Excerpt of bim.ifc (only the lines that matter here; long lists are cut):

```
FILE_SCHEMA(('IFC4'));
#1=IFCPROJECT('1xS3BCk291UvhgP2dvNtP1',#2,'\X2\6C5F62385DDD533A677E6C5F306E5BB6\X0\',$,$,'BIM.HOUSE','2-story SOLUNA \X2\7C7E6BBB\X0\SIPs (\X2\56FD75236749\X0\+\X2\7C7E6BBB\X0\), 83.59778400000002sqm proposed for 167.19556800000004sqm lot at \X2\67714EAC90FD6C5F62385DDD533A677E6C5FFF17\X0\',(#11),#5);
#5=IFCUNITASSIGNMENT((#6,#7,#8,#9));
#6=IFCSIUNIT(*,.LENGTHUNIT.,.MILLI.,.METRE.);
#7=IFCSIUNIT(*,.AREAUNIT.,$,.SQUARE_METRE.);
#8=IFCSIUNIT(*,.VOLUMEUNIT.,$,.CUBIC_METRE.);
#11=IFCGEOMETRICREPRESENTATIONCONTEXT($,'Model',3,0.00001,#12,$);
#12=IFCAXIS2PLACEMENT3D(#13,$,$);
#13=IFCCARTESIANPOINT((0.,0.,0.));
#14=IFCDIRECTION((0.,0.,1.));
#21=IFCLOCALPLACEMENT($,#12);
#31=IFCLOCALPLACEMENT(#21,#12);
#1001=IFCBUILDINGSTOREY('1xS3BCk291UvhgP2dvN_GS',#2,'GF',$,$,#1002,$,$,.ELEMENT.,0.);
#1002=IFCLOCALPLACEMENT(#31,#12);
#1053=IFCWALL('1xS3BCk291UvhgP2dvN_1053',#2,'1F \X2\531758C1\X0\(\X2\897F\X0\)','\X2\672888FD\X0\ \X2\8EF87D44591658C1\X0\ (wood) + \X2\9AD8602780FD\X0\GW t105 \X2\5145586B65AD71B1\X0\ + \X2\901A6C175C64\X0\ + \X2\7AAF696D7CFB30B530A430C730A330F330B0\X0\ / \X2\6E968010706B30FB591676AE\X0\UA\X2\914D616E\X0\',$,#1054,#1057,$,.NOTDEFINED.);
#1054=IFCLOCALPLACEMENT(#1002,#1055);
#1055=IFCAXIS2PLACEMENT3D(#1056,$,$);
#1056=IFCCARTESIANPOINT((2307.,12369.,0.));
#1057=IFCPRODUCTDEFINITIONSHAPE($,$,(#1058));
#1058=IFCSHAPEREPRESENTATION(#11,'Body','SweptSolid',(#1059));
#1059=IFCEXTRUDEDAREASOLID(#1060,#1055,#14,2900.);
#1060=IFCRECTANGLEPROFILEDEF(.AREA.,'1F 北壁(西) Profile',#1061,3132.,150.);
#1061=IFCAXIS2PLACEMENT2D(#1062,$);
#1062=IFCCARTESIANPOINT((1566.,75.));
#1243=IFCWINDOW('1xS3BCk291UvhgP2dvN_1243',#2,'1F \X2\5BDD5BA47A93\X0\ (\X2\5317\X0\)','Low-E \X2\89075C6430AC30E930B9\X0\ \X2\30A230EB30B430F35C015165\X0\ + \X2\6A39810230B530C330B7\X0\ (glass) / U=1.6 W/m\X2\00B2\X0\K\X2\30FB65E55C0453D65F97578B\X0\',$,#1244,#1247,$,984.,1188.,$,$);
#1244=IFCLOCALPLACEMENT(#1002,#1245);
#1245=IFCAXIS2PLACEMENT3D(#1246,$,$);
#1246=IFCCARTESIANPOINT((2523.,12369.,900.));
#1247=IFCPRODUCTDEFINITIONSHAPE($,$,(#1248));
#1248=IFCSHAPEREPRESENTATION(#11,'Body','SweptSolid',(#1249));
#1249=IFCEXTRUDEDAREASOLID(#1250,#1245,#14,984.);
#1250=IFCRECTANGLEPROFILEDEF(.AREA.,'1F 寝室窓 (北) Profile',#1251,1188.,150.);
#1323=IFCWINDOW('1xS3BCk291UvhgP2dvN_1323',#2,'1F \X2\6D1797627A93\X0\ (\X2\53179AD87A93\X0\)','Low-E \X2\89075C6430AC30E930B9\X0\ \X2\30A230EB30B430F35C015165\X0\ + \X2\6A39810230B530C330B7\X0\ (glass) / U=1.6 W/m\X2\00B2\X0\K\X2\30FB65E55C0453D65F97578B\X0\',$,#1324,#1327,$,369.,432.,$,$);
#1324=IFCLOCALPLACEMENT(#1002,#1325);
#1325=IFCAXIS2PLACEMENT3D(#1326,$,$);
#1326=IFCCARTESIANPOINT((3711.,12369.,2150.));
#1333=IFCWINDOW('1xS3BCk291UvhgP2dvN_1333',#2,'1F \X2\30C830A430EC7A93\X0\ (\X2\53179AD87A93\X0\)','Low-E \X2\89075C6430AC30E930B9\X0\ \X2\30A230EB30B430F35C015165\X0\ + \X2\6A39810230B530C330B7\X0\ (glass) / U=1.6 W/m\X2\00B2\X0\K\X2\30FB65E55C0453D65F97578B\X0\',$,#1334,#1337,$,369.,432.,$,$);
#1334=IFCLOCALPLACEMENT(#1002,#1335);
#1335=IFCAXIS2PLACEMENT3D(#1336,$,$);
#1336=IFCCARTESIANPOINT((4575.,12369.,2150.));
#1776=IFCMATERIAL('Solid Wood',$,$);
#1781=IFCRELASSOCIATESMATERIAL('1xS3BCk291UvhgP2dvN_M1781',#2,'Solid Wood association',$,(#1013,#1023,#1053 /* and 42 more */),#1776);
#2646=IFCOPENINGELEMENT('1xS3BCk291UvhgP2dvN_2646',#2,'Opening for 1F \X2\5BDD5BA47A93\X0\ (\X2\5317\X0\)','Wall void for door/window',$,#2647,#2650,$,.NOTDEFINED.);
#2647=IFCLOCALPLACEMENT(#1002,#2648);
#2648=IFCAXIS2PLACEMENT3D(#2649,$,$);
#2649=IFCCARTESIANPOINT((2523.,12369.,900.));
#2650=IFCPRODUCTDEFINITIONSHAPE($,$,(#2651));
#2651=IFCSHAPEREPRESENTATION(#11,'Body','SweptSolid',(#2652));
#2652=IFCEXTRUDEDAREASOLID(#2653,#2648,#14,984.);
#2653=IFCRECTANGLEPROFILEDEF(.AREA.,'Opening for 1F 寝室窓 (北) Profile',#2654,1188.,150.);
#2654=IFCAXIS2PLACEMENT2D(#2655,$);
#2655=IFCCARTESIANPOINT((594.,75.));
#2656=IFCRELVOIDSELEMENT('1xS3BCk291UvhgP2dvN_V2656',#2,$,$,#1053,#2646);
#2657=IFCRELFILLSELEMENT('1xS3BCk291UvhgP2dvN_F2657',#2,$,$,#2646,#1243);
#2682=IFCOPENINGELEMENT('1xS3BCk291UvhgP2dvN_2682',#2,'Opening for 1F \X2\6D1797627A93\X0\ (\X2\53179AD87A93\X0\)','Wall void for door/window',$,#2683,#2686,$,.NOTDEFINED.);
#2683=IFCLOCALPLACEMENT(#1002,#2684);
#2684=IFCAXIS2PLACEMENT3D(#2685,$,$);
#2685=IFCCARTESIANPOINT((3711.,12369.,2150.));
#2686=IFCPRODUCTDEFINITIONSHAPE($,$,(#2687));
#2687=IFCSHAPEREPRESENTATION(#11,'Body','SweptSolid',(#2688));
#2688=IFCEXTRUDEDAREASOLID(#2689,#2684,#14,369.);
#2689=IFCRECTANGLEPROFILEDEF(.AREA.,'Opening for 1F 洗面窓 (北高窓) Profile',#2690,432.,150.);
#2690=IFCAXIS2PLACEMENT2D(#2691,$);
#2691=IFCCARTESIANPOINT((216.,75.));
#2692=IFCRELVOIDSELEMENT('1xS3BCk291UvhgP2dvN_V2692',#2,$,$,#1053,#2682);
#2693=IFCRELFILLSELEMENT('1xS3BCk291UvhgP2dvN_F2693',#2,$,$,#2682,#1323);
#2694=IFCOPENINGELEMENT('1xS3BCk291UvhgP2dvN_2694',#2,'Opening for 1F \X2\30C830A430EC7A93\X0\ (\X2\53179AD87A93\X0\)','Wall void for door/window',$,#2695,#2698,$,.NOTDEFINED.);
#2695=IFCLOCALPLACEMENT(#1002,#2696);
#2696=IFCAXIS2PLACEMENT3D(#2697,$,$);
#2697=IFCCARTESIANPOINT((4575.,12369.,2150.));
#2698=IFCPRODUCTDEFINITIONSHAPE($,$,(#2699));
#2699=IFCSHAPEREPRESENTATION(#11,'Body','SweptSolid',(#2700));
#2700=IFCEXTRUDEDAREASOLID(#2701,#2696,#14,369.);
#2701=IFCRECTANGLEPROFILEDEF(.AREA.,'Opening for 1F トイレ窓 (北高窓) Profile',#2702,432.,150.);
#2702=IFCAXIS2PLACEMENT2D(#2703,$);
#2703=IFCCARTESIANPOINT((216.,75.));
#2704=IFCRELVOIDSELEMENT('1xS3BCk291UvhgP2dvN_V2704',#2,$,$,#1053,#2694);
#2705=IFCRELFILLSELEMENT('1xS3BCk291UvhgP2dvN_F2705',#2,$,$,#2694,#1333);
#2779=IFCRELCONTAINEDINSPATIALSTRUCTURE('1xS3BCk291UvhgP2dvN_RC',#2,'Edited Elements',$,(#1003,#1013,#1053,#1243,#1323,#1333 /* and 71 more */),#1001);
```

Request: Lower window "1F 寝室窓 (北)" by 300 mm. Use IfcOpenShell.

```python
import numpy as np
import ifcopenshell
import ifcopenshell.api.geometry
import ifcopenshell.util.placement
import ifcopenshell.util.unit

model = ifcopenshell.open("bim.ifc")
unit_scale = ifcopenshell.util.unit.calculate_unit_scale(model)

window = model.by_guid("1xS3BCk291UvhgP2dvN_1243")
opening = window.FillsVoids[0].RelatingOpeningElement
dz = -300.0

shift = np.array([0.0, 0.0, dz])
# The window is not placed relative to its opening, so move both.
for product in (opening, window):
    matrix = ifcopenshell.util.placement.get_local_placement(product.ObjectPlacement)
    matrix[:3, 3] += shift
    ifcopenshell.api.geometry.edit_object_placement(model, product=product, matrix=matrix, is_si=False)

print(f"moved by {dz * unit_scale:+.3f} m")

model.write("bim_rev.ifc")
```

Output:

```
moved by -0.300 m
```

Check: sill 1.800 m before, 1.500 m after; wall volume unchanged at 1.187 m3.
